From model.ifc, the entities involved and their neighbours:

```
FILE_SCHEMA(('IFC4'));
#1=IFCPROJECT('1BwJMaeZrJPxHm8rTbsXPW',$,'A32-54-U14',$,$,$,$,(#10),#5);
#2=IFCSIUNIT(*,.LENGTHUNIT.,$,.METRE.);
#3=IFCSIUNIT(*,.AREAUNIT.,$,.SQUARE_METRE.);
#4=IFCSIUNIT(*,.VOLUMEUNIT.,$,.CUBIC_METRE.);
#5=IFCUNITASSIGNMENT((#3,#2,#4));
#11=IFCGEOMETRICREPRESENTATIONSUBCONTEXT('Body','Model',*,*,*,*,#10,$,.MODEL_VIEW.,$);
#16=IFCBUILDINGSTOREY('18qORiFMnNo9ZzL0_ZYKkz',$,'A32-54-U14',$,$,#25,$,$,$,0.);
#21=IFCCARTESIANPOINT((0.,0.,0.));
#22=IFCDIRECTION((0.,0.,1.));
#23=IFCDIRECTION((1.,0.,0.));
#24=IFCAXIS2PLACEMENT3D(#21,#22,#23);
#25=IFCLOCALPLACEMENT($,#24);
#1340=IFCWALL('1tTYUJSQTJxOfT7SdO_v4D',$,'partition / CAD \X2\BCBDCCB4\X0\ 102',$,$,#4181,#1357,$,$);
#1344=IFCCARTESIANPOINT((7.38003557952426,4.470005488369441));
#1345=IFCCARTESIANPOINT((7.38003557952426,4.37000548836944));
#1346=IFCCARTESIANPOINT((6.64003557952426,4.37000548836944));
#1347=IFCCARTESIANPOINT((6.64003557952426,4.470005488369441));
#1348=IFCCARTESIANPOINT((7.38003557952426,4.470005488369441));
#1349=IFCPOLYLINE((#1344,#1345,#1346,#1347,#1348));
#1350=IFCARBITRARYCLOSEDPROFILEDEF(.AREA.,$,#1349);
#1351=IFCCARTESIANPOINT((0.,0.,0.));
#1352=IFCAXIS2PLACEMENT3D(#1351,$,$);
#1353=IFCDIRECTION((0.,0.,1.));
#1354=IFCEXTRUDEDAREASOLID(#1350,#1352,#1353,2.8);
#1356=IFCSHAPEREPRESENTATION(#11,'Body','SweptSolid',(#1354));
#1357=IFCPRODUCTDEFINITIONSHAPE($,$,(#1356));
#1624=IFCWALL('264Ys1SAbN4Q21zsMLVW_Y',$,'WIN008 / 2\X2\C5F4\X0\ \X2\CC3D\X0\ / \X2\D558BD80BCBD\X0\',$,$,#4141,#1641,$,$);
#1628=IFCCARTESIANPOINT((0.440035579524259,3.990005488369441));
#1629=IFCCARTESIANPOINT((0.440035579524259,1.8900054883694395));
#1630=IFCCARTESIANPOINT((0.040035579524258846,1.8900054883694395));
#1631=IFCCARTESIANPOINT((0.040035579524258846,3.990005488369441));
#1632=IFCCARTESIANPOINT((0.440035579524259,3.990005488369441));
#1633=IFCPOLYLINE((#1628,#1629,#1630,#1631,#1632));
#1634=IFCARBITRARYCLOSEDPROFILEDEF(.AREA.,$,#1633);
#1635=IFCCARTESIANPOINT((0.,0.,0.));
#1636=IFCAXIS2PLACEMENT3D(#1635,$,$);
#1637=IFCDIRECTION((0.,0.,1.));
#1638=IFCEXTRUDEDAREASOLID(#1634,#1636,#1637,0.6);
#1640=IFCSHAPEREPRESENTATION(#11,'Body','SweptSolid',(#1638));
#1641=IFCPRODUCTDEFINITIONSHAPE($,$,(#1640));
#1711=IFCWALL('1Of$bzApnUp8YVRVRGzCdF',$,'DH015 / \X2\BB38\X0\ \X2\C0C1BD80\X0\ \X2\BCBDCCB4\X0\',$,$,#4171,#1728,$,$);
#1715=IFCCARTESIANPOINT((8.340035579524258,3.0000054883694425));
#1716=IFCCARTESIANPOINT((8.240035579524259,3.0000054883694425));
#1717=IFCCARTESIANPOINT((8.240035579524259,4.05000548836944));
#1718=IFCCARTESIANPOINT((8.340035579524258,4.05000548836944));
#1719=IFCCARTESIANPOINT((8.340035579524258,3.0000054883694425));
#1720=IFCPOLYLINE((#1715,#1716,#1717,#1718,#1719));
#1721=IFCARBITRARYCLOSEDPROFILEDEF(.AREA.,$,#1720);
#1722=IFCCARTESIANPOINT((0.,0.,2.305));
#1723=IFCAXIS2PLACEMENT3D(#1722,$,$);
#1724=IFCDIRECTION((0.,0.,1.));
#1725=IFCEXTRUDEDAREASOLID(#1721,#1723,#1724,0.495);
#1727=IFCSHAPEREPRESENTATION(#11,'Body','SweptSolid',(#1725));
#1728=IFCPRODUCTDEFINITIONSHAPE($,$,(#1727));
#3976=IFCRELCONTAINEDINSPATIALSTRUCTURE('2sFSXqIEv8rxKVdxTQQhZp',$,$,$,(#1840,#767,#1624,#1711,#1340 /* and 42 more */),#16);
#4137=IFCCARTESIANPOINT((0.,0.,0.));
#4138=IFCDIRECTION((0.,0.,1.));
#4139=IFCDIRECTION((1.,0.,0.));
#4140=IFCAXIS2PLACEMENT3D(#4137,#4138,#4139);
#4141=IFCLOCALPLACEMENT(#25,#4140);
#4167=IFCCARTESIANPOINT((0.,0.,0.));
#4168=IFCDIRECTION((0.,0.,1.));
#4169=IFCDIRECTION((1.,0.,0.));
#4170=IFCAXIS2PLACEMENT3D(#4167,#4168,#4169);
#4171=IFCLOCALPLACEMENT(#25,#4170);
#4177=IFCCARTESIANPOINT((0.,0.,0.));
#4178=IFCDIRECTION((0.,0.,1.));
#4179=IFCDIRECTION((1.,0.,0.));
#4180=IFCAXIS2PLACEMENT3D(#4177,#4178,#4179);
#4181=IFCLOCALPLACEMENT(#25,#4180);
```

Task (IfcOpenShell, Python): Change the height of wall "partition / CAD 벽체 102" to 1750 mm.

```python
import ifcopenshell
import ifcopenshell.geom
import ifcopenshell.util.representation
import ifcopenshell.util.shape
import ifcopenshell.util.unit

model = ifcopenshell.open("model.ifc")
unit_scale = ifcopenshell.util.unit.calculate_unit_scale(model)
settings = ifcopenshell.geom.settings()


def volume(element):
    """Net volume in cubic metres, openings subtracted."""
    shape = ifcopenshell.geom.create_shape(settings, element)
    return ifcopenshell.util.shape.get_volume(shape.geometry)


wall = model.by_guid("1tTYUJSQTJxOfT7SdO_v4D")
before = volume(wall)

body = ifcopenshell.util.representation.get_representation(wall, "Model", "Body")
solid = body.Items[0]
old_height = solid.Depth
solid.Depth = 1.75 / unit_scale
after = volume(wall)

print(f"height {old_height:g} -> {solid.Depth:g}, volume {before:.3f} -> {after:.3f} m3")

model.write("model-out.ifc")
```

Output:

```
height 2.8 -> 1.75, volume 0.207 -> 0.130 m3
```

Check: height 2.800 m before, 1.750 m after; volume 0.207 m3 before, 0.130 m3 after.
